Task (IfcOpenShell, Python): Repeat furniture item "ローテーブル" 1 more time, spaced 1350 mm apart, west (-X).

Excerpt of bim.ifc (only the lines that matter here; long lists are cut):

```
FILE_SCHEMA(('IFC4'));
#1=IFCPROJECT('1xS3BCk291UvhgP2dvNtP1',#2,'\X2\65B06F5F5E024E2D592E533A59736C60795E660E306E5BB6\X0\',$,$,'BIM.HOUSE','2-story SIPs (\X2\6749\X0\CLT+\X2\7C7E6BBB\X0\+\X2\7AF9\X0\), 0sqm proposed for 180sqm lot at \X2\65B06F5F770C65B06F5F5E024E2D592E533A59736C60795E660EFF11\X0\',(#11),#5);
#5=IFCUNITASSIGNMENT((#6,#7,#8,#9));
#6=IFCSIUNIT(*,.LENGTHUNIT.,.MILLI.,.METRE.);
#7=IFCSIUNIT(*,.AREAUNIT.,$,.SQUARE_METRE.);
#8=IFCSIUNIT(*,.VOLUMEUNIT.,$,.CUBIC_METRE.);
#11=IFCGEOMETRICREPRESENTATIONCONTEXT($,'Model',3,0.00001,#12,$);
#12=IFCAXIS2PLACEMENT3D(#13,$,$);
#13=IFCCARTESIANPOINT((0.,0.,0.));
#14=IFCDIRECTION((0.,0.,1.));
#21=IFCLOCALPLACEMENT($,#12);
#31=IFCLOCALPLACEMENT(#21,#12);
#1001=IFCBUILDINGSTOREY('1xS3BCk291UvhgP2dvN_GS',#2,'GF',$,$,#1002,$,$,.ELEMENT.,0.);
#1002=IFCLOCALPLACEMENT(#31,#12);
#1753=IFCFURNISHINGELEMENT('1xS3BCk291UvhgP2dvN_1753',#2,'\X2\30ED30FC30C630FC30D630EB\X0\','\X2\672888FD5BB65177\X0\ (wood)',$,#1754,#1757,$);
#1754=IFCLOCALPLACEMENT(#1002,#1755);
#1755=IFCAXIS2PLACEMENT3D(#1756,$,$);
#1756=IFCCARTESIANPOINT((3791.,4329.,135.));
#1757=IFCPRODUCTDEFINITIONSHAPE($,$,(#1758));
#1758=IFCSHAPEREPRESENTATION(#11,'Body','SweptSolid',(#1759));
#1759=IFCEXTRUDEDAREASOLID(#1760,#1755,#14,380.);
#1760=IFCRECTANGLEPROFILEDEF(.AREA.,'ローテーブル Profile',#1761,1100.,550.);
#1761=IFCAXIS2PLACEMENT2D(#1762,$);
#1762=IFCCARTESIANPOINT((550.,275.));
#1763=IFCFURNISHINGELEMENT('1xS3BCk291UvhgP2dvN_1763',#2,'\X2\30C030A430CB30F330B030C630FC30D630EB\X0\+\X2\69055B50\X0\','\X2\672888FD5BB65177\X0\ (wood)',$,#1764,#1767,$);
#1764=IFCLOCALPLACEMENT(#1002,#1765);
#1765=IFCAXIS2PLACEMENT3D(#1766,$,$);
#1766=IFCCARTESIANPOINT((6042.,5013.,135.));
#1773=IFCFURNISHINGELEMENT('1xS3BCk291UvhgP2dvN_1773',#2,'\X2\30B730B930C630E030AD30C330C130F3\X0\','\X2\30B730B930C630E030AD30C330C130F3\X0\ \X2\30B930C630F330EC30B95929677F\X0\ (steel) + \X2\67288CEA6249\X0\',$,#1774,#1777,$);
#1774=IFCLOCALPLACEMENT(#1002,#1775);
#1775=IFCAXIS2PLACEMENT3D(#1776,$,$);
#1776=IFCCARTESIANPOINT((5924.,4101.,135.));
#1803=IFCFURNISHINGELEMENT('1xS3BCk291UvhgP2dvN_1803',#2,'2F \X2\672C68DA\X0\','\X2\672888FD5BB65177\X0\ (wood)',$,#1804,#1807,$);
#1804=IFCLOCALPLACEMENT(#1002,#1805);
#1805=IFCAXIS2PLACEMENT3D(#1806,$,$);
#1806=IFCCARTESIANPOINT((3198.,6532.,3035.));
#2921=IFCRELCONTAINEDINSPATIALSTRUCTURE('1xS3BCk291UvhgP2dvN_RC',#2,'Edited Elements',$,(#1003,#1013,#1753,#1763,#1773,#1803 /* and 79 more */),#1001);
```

```python
import numpy as np
import ifcopenshell
import ifcopenshell.api.geometry
import ifcopenshell.api.root
import ifcopenshell.util.element
import ifcopenshell.util.placement
import ifcopenshell.util.unit

model = ifcopenshell.open("bim.ifc")
unit_scale = ifcopenshell.util.unit.calculate_unit_scale(model)


def reuse_history(source, copy):
    """copy_class also copies each property set's owner history, people and application; keep the originals."""
    for rel in copy.IsDefinedBy:
        if rel.is_a("IfcRelDefinesByProperties") and (history := rel.RelatingPropertyDefinition.OwnerHistory):
            rel.RelatingPropertyDefinition.OwnerHistory = source.OwnerHistory
            ifcopenshell.util.element.remove_deep2(model, history)


source = model.by_id(1753)
base = ifcopenshell.util.placement.get_local_placement(source.ObjectPlacement)
step = np.array([-1.0, 0.0, 0.0]) * 1.35 / unit_scale

for i in range(1, 2):
    copy = ifcopenshell.api.root.copy_class(model, product=source)
    copy.Representation = ifcopenshell.util.element.copy_deep(
        model, source.Representation, exclude=["IfcGeometricRepresentationContext", "IfcRepresentationMap"]
    )
    reuse_history(source, copy)
    matrix = base.copy()
    matrix[:3, 3] += i * step
    print("added at", matrix[:3, 3].round(3) + 0.0)
    ifcopenshell.api.geometry.edit_object_placement(model, product=copy, matrix=matrix, is_si=False)

model.write("bim_updated.ifc")
```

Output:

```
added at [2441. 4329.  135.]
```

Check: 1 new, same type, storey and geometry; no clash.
